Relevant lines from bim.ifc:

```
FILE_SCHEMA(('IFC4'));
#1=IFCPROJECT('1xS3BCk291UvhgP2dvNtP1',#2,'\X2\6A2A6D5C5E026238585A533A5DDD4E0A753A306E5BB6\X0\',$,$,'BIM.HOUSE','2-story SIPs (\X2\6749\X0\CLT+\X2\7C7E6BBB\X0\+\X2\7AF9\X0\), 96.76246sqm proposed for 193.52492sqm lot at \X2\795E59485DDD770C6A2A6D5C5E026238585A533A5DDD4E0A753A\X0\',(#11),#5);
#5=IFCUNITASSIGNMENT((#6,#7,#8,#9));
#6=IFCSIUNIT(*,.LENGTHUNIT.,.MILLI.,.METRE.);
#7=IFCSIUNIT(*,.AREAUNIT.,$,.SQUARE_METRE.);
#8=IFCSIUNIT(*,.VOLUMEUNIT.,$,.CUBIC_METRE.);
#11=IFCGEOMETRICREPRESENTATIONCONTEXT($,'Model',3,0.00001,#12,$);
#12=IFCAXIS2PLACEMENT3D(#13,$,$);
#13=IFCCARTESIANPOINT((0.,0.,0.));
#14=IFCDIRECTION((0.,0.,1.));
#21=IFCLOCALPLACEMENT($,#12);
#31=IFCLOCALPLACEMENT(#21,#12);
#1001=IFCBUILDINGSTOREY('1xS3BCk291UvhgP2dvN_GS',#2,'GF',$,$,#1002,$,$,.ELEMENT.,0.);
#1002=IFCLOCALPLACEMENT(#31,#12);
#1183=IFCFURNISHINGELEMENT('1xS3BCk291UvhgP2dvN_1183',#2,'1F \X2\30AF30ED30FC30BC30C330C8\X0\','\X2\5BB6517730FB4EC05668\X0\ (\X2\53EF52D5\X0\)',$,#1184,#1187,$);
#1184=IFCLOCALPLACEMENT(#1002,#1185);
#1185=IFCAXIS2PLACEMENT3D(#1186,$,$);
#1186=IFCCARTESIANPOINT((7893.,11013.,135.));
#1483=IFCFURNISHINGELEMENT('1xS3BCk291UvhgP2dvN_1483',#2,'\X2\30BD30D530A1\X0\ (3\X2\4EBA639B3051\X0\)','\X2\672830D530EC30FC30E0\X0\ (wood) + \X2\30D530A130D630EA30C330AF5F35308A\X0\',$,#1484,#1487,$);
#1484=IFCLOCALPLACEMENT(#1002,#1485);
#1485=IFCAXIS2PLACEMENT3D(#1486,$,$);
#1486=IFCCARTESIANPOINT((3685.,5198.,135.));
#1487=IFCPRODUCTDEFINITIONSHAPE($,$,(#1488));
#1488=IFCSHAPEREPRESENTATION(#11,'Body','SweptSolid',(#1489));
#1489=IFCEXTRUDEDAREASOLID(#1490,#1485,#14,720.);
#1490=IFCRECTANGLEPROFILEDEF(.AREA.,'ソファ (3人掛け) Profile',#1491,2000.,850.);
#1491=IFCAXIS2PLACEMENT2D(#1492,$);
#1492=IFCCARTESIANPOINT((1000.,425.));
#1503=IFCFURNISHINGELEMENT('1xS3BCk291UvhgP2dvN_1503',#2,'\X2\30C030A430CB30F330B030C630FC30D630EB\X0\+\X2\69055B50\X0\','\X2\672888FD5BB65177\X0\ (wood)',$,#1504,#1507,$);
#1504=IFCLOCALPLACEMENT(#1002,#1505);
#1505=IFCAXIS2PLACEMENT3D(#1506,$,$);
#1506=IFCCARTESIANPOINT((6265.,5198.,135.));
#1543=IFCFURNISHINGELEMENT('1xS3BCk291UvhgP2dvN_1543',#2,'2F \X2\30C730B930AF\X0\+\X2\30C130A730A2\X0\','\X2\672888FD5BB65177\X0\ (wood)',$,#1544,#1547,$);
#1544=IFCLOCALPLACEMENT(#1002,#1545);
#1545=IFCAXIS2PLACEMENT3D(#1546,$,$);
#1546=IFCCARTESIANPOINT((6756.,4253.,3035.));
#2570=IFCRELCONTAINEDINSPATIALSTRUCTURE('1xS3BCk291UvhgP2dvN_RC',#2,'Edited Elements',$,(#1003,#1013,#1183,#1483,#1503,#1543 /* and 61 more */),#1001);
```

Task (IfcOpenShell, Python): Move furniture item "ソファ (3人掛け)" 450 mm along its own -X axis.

```python
import ifcopenshell
import ifcopenshell.api.geometry
import ifcopenshell.util.placement
import ifcopenshell.util.unit

model = ifcopenshell.open("bim.ifc")
unit_scale = ifcopenshell.util.unit.calculate_unit_scale(model)

item = model.by_guid("1xS3BCk291UvhgP2dvN_1483")
matrix = ifcopenshell.util.placement.get_local_placement(item.ObjectPlacement)
matrix[:3, 3] -= matrix[:3, 0] * 0.45 / unit_scale
ifcopenshell.api.geometry.edit_object_placement(model, product=item, matrix=matrix, is_si=False)

print(ifcopenshell.util.placement.get_local_placement(item.ObjectPlacement).round(3) + 0.0)

model.write("bim_v2.ifc")
```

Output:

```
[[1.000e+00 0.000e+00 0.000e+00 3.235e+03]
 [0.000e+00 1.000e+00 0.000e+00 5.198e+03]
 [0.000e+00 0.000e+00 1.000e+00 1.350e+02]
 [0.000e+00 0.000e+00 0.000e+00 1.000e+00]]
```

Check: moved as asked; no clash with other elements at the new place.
